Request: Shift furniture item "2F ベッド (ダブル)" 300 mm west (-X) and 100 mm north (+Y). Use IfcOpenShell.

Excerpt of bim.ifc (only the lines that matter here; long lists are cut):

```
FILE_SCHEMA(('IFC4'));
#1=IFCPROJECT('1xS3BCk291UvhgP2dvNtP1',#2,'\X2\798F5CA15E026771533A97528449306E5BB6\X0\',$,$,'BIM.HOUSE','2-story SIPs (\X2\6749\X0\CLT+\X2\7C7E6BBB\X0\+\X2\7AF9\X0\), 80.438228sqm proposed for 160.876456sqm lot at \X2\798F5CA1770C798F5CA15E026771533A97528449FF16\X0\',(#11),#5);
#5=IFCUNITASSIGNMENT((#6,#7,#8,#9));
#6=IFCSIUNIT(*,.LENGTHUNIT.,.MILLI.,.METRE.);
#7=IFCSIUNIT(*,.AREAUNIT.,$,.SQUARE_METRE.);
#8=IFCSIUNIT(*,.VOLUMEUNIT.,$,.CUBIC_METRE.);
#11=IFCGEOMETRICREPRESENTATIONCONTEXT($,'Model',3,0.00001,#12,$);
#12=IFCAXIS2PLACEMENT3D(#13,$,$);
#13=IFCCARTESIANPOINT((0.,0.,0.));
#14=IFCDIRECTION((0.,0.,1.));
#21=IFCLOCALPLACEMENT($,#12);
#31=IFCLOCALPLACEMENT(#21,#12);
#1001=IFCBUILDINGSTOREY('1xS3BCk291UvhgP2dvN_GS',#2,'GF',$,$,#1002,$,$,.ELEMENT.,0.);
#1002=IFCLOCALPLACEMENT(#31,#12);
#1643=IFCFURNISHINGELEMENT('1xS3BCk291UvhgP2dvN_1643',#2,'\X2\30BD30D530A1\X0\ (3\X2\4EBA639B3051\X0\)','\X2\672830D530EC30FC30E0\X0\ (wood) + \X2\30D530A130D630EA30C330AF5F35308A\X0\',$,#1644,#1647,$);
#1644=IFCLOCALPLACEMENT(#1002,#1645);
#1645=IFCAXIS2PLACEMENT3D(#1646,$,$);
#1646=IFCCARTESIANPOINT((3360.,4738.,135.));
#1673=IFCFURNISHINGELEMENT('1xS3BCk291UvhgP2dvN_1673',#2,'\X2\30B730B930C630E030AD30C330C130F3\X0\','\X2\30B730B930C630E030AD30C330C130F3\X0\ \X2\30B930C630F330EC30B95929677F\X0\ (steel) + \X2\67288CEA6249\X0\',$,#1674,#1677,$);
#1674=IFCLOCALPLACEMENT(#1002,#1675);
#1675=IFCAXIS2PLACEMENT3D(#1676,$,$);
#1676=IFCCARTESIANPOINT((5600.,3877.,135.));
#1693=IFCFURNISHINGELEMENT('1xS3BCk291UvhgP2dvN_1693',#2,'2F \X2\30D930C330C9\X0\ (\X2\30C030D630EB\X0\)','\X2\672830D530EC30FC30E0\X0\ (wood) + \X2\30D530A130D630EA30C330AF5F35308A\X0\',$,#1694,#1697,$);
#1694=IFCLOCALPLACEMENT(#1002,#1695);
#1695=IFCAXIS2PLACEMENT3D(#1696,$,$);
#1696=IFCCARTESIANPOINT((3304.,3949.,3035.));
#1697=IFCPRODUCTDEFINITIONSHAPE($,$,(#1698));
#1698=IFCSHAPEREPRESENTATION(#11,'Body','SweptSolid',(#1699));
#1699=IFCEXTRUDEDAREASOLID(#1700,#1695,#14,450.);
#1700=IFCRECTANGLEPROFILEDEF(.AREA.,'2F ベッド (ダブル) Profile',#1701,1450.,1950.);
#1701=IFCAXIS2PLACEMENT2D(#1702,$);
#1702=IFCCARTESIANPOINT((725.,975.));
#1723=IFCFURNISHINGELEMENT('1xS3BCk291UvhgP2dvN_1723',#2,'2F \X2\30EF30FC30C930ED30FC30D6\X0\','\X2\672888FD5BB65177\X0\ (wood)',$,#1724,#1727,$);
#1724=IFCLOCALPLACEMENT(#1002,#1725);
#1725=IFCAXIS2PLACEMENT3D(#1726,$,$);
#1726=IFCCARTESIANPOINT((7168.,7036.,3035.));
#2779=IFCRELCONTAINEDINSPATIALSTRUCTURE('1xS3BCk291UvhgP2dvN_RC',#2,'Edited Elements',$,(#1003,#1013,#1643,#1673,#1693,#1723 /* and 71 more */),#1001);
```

```python
import ifcopenshell
import ifcopenshell.api.geometry
import ifcopenshell.util.placement
import ifcopenshell.util.unit

model = ifcopenshell.open("bim.ifc")
unit_scale = ifcopenshell.util.unit.calculate_unit_scale(model)

item = model.by_guid("1xS3BCk291UvhgP2dvN_1693")
matrix = ifcopenshell.util.placement.get_local_placement(item.ObjectPlacement)
matrix[0, 3] -= 0.3 / unit_scale
matrix[1, 3] += 0.1 / unit_scale
ifcopenshell.api.geometry.edit_object_placement(model, product=item, matrix=matrix, is_si=False)

print(ifcopenshell.util.placement.get_local_placement(item.ObjectPlacement).round(3) + 0.0)

model.write("bim_v2.ifc")
```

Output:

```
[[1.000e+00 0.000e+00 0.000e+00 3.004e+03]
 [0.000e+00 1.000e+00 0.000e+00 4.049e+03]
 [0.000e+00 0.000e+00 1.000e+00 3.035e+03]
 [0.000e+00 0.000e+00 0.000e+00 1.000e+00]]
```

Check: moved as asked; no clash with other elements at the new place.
